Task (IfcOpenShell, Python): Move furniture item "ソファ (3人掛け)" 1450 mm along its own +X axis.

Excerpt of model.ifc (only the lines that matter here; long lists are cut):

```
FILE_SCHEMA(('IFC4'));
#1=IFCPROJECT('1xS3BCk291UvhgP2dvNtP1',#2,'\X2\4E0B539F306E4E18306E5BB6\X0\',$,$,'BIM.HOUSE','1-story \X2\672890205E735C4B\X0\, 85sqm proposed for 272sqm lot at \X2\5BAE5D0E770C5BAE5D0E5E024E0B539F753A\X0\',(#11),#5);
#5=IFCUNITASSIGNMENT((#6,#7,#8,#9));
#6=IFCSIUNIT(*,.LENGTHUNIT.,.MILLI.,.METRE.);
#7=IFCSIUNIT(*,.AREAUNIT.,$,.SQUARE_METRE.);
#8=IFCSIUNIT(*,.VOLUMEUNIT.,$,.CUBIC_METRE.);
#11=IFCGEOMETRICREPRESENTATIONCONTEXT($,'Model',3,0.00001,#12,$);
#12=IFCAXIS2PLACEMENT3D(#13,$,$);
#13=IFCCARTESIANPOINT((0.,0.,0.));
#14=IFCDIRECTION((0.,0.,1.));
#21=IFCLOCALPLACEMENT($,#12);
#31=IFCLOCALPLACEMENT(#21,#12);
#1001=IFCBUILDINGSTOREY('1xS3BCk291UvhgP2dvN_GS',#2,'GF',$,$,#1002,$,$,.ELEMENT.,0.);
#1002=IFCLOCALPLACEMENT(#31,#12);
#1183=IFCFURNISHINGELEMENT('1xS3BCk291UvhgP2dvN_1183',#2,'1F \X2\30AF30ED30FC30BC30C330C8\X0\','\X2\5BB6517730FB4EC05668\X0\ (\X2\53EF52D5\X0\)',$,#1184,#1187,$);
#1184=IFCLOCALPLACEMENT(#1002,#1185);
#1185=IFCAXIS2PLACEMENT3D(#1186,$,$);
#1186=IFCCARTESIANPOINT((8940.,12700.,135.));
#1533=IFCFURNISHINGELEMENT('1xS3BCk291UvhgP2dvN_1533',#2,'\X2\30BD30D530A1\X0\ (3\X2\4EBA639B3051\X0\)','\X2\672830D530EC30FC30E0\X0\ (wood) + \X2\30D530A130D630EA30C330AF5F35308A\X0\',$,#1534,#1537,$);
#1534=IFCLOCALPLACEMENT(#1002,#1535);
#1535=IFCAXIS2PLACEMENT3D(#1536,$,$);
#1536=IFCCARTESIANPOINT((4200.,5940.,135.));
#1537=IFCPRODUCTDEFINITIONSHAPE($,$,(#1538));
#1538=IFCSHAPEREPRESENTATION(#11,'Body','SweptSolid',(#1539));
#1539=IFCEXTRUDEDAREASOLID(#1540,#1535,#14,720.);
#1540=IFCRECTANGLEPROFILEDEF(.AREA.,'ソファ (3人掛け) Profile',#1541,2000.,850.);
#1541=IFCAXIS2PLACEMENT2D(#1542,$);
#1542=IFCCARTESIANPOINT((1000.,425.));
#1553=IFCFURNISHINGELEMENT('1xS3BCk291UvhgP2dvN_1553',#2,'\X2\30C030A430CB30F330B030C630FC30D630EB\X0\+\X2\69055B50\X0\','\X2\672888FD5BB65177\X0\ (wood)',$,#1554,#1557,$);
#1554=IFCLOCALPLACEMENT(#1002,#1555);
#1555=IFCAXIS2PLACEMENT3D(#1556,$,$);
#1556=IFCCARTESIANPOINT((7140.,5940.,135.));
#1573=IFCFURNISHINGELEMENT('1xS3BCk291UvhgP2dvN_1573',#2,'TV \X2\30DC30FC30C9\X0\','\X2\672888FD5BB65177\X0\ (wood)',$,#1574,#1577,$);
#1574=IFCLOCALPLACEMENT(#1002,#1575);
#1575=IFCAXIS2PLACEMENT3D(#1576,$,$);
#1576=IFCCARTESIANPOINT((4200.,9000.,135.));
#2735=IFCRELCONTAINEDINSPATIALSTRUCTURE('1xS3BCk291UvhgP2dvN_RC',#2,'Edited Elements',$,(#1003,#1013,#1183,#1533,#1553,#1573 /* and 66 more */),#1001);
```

```python
import ifcopenshell
import ifcopenshell.api.geometry
import ifcopenshell.util.placement

model = ifcopenshell.open("model.ifc")

item = model.by_guid("1xS3BCk291UvhgP2dvN_1533")
matrix = ifcopenshell.util.placement.get_local_placement(item.ObjectPlacement)
matrix[:3, 3] += matrix[:3, 0] * 1450.0
ifcopenshell.api.geometry.edit_object_placement(model, product=item, matrix=matrix, is_si=False)

print(ifcopenshell.util.placement.get_local_placement(item.ObjectPlacement).round(3) + 0.0)

model.write("model-out.ifc")
```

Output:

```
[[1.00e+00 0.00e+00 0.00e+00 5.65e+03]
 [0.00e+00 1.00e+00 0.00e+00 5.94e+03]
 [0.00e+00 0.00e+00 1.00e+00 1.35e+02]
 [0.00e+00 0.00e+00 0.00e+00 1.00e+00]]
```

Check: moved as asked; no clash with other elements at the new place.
